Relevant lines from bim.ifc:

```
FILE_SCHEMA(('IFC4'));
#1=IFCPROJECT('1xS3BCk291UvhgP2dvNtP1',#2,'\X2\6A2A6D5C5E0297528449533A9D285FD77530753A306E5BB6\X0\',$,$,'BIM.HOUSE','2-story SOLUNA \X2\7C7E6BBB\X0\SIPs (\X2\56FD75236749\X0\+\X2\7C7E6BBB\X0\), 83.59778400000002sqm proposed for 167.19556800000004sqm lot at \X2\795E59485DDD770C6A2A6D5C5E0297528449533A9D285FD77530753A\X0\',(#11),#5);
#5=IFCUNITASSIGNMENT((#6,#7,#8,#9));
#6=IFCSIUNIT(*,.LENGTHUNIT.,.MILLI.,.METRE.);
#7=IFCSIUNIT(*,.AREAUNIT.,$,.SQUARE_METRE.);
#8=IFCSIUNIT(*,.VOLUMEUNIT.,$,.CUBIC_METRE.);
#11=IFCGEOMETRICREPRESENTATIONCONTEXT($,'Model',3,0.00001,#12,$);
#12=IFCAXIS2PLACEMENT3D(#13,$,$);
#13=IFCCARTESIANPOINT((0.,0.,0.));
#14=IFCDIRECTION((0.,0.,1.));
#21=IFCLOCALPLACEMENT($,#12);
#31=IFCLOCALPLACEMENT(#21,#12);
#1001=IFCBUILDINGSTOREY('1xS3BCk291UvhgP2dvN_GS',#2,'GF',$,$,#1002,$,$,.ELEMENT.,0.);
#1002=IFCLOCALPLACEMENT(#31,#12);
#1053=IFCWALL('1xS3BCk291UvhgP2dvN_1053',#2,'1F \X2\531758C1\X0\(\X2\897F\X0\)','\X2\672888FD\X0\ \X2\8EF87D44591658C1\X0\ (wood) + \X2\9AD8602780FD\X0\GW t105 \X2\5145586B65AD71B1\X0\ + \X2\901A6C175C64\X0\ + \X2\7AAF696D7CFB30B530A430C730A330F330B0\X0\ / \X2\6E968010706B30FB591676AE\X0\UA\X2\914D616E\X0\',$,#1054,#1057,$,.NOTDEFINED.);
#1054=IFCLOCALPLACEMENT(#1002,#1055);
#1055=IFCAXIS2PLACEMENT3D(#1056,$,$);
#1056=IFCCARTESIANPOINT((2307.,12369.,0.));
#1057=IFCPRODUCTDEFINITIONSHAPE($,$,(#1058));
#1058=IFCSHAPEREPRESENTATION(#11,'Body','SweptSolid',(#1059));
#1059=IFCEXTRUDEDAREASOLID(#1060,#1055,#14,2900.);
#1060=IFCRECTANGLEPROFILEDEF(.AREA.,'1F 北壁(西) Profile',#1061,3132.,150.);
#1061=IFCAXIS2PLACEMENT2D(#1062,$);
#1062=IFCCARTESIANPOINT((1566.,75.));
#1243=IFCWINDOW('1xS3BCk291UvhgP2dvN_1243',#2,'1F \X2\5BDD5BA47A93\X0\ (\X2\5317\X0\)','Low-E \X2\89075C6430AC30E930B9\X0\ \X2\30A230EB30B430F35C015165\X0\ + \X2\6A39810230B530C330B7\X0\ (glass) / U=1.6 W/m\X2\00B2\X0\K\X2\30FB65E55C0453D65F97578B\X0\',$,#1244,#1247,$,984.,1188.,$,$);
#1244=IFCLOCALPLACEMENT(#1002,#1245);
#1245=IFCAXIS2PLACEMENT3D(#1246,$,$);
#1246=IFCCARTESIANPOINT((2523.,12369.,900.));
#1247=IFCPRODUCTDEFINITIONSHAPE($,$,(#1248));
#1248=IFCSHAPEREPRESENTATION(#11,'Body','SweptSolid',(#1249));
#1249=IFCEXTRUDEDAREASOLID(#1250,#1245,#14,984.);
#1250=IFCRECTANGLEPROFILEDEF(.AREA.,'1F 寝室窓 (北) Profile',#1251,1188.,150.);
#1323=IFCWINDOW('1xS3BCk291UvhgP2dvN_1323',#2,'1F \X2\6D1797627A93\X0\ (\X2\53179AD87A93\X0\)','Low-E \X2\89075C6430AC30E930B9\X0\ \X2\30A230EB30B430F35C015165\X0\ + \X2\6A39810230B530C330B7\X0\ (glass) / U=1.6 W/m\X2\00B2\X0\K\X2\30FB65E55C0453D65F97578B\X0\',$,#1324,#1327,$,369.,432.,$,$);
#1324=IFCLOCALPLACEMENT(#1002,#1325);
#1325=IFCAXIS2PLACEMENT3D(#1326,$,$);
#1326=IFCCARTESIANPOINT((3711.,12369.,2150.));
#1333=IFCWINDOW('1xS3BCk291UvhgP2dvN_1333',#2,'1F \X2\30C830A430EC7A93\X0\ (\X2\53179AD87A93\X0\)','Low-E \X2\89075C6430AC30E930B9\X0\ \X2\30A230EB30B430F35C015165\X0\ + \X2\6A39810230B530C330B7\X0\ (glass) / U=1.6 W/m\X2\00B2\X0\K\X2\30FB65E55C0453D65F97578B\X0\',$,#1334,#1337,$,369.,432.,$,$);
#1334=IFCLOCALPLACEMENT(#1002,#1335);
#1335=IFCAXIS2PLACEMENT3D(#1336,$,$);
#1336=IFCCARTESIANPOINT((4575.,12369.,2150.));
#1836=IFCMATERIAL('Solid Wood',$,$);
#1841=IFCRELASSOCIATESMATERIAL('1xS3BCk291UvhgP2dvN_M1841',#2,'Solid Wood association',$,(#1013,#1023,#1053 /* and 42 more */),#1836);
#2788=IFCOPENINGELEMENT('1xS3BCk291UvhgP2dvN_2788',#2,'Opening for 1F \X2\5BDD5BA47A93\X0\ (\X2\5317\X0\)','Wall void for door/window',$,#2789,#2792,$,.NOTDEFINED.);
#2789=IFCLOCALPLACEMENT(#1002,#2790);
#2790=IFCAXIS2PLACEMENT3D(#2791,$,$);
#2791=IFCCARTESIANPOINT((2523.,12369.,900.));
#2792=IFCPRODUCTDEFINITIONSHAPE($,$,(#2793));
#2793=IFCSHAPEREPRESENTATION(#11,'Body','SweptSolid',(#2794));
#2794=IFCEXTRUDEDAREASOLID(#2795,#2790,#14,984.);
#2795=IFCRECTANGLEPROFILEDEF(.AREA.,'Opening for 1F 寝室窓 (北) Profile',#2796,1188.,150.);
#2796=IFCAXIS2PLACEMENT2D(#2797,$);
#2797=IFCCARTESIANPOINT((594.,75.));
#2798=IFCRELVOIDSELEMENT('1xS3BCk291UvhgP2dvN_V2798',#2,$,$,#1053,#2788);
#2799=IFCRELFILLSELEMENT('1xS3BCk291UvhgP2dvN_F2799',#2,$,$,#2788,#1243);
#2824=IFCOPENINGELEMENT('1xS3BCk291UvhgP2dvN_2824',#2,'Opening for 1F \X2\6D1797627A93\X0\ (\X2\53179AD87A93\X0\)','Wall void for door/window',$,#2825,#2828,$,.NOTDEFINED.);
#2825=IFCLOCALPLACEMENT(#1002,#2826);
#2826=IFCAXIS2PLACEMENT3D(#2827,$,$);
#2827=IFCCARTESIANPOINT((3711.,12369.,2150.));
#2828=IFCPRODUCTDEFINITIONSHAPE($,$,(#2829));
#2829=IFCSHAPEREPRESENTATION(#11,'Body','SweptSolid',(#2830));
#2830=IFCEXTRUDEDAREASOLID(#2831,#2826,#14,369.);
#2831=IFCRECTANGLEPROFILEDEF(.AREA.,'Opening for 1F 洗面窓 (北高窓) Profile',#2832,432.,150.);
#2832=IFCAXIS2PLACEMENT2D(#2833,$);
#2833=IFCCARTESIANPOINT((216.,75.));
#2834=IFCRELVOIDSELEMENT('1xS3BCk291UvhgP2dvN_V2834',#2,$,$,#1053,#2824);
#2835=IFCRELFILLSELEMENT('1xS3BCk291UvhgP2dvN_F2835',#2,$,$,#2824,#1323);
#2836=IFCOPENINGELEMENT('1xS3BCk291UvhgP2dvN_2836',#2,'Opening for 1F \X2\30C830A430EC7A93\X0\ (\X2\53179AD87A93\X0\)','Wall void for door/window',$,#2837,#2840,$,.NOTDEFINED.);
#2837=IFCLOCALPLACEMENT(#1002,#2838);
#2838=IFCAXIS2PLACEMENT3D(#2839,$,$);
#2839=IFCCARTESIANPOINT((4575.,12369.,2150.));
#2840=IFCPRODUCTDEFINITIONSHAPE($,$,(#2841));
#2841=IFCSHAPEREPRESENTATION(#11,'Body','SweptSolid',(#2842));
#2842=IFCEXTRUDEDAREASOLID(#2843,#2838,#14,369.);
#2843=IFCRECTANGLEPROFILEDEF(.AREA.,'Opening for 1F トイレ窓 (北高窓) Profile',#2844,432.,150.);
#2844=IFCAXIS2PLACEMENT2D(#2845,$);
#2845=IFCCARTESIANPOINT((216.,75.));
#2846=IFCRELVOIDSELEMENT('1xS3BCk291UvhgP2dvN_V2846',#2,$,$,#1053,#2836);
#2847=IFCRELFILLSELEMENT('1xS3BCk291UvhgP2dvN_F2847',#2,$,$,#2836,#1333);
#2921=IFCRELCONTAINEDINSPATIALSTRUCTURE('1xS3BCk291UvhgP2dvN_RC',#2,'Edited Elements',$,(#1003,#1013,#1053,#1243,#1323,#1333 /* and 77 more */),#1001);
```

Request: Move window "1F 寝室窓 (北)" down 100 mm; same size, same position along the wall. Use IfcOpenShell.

```python
import numpy as np
import ifcopenshell
import ifcopenshell.api.geometry
import ifcopenshell.util.placement
import ifcopenshell.util.unit

model = ifcopenshell.open("bim.ifc")
unit_scale = ifcopenshell.util.unit.calculate_unit_scale(model)

window = model.by_guid("1xS3BCk291UvhgP2dvN_1243")
opening = window.FillsVoids[0].RelatingOpeningElement
dz = -0.1 / unit_scale

shift = np.array([0.0, 0.0, dz])
# The window is not placed relative to its opening, so move both.
for product in (opening, window):
    matrix = ifcopenshell.util.placement.get_local_placement(product.ObjectPlacement)
    matrix[:3, 3] += shift
    ifcopenshell.api.geometry.edit_object_placement(model, product=product, matrix=matrix, is_si=False)

print(f"moved by {dz * unit_scale:+.3f} m")

model.write("bim_updated.ifc")
```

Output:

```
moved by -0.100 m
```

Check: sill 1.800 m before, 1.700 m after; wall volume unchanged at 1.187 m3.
